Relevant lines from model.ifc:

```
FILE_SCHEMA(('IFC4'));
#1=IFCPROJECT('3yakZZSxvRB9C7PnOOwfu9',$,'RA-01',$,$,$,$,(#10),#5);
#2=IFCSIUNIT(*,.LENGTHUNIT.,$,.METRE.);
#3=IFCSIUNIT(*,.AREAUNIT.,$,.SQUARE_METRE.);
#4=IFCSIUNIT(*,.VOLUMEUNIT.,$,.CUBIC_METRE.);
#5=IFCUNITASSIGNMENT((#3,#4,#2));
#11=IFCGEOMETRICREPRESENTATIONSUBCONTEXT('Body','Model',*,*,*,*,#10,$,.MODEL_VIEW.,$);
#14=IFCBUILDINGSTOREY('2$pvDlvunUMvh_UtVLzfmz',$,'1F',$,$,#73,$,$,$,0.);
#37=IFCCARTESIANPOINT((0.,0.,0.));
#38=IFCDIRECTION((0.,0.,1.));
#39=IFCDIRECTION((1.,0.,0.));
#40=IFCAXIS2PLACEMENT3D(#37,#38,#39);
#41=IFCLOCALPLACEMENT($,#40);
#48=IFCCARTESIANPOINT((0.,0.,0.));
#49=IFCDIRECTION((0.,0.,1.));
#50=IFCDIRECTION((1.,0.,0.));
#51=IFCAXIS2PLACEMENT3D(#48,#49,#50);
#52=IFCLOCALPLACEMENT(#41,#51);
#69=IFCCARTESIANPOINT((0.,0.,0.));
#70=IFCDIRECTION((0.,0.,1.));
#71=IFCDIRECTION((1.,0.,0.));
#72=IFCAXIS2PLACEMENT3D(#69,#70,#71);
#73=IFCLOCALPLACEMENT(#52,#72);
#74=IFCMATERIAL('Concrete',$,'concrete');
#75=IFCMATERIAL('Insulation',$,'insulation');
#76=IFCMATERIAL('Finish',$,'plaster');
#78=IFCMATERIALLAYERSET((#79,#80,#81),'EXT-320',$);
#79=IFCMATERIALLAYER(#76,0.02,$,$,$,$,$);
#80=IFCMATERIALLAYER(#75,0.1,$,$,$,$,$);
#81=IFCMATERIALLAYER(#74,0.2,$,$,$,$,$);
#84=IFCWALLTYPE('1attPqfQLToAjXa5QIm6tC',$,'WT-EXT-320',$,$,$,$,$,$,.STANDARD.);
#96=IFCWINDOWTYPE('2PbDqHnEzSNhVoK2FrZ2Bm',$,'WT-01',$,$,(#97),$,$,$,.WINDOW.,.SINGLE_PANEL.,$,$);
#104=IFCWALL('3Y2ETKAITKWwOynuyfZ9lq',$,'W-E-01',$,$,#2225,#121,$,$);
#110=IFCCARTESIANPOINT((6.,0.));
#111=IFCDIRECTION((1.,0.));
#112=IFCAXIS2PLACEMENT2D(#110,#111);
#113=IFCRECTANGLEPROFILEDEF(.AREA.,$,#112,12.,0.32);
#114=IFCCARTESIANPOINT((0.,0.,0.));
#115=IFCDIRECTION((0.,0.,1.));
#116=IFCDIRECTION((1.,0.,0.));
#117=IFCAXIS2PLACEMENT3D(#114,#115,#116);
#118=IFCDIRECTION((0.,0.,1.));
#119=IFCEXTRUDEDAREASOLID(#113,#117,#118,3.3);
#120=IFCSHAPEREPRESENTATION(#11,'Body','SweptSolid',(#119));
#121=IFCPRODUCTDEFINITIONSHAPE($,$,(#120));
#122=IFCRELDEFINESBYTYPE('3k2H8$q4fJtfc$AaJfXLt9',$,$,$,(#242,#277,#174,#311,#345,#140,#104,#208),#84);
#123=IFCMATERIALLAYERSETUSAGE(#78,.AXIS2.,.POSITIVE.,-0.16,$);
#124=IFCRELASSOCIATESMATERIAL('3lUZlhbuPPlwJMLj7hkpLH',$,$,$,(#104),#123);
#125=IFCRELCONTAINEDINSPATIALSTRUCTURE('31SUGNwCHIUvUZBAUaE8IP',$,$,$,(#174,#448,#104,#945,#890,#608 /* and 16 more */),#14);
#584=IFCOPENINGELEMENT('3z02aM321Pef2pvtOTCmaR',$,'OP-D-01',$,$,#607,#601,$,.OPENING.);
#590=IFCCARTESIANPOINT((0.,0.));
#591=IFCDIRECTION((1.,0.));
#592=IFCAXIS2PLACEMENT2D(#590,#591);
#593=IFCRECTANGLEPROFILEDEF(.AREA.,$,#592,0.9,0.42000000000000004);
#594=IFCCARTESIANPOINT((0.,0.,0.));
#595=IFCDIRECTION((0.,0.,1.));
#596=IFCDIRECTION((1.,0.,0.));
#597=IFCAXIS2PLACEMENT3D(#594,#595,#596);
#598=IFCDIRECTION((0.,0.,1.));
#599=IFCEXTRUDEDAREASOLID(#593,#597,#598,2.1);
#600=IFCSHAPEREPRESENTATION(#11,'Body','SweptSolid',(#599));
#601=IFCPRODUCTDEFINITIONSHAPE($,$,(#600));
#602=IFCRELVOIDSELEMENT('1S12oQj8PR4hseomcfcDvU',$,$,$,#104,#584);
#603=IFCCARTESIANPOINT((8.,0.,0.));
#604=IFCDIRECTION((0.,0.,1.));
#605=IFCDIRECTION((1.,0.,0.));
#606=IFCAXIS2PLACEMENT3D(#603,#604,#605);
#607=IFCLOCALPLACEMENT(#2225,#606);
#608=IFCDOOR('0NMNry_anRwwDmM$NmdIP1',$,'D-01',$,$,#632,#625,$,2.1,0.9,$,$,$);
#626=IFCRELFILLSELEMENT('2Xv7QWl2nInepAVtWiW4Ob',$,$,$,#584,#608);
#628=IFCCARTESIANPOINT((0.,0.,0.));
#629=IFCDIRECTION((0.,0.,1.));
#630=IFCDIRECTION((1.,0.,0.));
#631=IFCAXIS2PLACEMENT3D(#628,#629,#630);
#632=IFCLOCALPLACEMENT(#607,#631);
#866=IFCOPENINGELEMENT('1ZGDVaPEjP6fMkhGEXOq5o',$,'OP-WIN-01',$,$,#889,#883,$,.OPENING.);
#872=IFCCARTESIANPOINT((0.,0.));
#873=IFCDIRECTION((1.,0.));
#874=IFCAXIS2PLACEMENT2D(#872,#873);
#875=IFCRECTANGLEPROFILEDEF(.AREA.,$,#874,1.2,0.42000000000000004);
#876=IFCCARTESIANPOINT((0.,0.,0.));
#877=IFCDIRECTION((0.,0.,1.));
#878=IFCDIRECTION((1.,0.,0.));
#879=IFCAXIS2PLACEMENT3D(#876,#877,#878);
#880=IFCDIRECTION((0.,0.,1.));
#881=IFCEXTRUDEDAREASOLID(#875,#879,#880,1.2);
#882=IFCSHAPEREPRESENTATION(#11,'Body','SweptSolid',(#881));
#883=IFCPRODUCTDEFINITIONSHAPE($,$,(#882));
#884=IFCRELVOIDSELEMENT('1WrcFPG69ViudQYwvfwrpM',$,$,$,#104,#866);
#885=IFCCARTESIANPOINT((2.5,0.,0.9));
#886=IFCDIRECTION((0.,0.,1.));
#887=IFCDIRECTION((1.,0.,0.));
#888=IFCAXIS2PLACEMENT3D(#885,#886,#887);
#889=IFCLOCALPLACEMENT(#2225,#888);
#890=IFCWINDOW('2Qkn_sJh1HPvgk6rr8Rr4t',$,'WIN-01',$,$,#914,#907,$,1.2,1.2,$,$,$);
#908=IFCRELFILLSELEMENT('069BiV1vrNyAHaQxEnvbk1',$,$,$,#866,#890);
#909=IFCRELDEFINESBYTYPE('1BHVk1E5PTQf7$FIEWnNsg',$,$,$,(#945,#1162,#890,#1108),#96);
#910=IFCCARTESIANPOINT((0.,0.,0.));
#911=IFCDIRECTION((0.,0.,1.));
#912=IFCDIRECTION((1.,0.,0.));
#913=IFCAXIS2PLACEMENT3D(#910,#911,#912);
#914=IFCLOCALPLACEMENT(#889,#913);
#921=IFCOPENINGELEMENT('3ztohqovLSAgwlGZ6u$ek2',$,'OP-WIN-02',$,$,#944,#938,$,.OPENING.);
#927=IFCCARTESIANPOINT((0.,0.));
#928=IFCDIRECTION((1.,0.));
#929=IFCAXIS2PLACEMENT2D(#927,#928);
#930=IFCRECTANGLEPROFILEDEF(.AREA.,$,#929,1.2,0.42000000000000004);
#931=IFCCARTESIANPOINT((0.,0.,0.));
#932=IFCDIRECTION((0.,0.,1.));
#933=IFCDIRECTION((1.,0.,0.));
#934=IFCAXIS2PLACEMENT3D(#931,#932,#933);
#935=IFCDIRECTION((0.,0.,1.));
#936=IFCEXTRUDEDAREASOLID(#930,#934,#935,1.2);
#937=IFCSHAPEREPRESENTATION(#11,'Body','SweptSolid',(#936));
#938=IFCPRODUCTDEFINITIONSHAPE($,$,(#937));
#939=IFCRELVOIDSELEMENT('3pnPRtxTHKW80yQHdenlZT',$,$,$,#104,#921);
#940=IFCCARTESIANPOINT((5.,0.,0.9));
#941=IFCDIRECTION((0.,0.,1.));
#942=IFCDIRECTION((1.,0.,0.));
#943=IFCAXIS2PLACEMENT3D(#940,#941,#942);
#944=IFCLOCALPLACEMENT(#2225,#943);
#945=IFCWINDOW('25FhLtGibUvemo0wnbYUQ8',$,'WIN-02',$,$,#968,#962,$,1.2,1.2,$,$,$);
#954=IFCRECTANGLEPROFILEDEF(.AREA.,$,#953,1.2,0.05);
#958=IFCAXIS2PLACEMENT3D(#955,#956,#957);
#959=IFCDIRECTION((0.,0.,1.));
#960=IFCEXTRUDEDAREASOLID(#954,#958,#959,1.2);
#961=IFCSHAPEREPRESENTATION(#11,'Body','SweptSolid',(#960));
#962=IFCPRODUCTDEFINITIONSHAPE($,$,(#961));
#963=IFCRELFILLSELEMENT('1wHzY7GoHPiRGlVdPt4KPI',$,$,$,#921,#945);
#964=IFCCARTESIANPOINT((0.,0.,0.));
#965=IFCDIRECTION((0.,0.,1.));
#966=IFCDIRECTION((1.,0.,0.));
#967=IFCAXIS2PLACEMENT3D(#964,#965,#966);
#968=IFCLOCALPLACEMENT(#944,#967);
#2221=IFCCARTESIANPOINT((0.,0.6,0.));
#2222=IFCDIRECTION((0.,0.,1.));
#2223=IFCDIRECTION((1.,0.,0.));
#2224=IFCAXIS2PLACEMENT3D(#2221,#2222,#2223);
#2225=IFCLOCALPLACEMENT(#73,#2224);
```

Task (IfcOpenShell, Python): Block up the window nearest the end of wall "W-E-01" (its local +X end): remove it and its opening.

```python
import ifcopenshell
import ifcopenshell.api.feature
import ifcopenshell.api.root
import ifcopenshell.geom
import ifcopenshell.util.shape

model = ifcopenshell.open("model.ifc")
settings = ifcopenshell.geom.settings()


def volume(element):
    """Net volume in cubic metres, openings subtracted."""
    shape = ifcopenshell.geom.create_shape(settings, element)
    return ifcopenshell.util.shape.get_volume(shape.geometry)


window = model.by_guid("25FhLtGibUvemo0wnbYUQ8")
opening = window.FillsVoids[0].RelatingOpeningElement
wall = opening.VoidsElements[0].RelatingBuildingElement
before = volume(wall)

ifcopenshell.api.root.remove_product(model, product=window)
ifcopenshell.api.feature.remove_feature(model, feature=opening)

after = volume(wall)

print(f"wall volume {before:.3f} -> {after:.3f} m3")

model.write("model-out.ifc")
```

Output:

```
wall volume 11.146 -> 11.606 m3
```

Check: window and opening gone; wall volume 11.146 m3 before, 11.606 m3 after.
